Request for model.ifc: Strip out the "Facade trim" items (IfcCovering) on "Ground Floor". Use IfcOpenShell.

First a look at what the model holds.

```python
import ifcopenshell
import ifcopenshell.util.element

model = ifcopenshell.open("model.ifc")
print(model.schema)
storey = next(s for s in model.by_type("IfcBuildingStorey") if s.Name == "Ground Floor")
coverings = [e for e in ifcopenshell.util.element.get_decomposition(storey) if e.is_a("IfcCovering")]
seen = {}
for e in coverings:
    element_type = ifcopenshell.util.element.get_type(e)
    name = element_type.Name if element_type not in (None, e) else None
    seen[name] = seen.get(name, 0) + 1
for name, count in sorted(seen.items(), key=str):
    print(count, "x", name)
```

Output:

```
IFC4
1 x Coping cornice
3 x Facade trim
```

```python
import ifcopenshell
import ifcopenshell.api.root
import ifcopenshell.util.element

model = ifcopenshell.open("model.ifc")

storey = next(s for s in model.by_type("IfcBuildingStorey") if s.Name == "Ground Floor")
coverings = [e for e in ifcopenshell.util.element.get_decomposition(storey) if e.is_a("IfcCovering")]
targets = [e for e in coverings if (t := ifcopenshell.util.element.get_type(e)) not in (None, e) and t.Name == "Facade trim"]

for e in targets:
    ifcopenshell.api.root.remove_product(model, product=e)
print(len(targets), "removed")

model.write("model_updated.ifc")
```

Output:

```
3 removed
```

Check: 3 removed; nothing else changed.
